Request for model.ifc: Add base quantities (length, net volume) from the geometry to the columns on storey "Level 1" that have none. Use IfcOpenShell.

First a look at what the model holds.

```python
import ifcopenshell
import ifcopenshell.util.element
import ifcopenshell.util.unit

model = ifcopenshell.open("model.ifc")
print(model.schema)
for unit_type in ("LENGTHUNIT", "AREAUNIT", "VOLUMEUNIT"):
    print(unit_type, ifcopenshell.util.unit.calculate_unit_scale(model, unit_type))
storey = next(s for s in model.by_type("IfcBuildingStorey") if s.Name == "Level 1")
columns = [e for e in ifcopenshell.util.element.get_decomposition(storey) if e.is_a("IfcColumn")]
for e in sorted(columns, key=lambda e: e.id()):
    print(e.id(), e.is_a(), e.Name, list(ifcopenshell.util.element.get_psets(e, qtos_only=True)), sep=" | ")
```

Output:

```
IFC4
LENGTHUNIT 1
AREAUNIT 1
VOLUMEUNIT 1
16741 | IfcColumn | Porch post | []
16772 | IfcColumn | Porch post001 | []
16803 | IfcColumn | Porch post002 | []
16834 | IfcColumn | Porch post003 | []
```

```python
import ifcopenshell
import ifcopenshell.api.pset
import ifcopenshell.geom
import ifcopenshell.util.element
import ifcopenshell.util.shape
import ifcopenshell.util.unit

model = ifcopenshell.open("model.ifc")
unit_scale = ifcopenshell.util.unit.calculate_unit_scale(model)
volume_scale = ifcopenshell.util.unit.calculate_unit_scale(model, "VOLUMEUNIT")
settings = ifcopenshell.geom.settings()

storey = next(s for s in model.by_type("IfcBuildingStorey") if s.Name == "Level 1")
columns = [e for e in ifcopenshell.util.element.get_decomposition(storey) if e.is_a("IfcColumn")]

for e in sorted(columns, key=lambda e: e.id()):
    if ifcopenshell.util.element.get_psets(e, qtos_only=True, should_inherit=False):
        continue
    # Geometry comes back in metres, in the element's own axes.
    shape = ifcopenshell.geom.create_shape(settings, e)
    values = {
        "Length": ifcopenshell.util.shape.get_z(shape.geometry) / unit_scale,
        "NetVolume": ifcopenshell.util.shape.get_volume(shape.geometry) / volume_scale,
    }
    qto = ifcopenshell.api.pset.add_qto(model, product=e, name="Qto_ColumnBaseQuantities")
    ifcopenshell.api.pset.edit_qto(model, qto=qto, properties=values)
    print(e.id(), {k: round(v, 3) for k, v in values.items()})

model.write("model-out.ifc")
```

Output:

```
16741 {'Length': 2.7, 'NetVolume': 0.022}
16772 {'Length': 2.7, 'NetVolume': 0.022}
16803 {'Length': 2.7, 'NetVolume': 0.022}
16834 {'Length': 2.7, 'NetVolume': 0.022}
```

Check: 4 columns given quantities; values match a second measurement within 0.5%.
